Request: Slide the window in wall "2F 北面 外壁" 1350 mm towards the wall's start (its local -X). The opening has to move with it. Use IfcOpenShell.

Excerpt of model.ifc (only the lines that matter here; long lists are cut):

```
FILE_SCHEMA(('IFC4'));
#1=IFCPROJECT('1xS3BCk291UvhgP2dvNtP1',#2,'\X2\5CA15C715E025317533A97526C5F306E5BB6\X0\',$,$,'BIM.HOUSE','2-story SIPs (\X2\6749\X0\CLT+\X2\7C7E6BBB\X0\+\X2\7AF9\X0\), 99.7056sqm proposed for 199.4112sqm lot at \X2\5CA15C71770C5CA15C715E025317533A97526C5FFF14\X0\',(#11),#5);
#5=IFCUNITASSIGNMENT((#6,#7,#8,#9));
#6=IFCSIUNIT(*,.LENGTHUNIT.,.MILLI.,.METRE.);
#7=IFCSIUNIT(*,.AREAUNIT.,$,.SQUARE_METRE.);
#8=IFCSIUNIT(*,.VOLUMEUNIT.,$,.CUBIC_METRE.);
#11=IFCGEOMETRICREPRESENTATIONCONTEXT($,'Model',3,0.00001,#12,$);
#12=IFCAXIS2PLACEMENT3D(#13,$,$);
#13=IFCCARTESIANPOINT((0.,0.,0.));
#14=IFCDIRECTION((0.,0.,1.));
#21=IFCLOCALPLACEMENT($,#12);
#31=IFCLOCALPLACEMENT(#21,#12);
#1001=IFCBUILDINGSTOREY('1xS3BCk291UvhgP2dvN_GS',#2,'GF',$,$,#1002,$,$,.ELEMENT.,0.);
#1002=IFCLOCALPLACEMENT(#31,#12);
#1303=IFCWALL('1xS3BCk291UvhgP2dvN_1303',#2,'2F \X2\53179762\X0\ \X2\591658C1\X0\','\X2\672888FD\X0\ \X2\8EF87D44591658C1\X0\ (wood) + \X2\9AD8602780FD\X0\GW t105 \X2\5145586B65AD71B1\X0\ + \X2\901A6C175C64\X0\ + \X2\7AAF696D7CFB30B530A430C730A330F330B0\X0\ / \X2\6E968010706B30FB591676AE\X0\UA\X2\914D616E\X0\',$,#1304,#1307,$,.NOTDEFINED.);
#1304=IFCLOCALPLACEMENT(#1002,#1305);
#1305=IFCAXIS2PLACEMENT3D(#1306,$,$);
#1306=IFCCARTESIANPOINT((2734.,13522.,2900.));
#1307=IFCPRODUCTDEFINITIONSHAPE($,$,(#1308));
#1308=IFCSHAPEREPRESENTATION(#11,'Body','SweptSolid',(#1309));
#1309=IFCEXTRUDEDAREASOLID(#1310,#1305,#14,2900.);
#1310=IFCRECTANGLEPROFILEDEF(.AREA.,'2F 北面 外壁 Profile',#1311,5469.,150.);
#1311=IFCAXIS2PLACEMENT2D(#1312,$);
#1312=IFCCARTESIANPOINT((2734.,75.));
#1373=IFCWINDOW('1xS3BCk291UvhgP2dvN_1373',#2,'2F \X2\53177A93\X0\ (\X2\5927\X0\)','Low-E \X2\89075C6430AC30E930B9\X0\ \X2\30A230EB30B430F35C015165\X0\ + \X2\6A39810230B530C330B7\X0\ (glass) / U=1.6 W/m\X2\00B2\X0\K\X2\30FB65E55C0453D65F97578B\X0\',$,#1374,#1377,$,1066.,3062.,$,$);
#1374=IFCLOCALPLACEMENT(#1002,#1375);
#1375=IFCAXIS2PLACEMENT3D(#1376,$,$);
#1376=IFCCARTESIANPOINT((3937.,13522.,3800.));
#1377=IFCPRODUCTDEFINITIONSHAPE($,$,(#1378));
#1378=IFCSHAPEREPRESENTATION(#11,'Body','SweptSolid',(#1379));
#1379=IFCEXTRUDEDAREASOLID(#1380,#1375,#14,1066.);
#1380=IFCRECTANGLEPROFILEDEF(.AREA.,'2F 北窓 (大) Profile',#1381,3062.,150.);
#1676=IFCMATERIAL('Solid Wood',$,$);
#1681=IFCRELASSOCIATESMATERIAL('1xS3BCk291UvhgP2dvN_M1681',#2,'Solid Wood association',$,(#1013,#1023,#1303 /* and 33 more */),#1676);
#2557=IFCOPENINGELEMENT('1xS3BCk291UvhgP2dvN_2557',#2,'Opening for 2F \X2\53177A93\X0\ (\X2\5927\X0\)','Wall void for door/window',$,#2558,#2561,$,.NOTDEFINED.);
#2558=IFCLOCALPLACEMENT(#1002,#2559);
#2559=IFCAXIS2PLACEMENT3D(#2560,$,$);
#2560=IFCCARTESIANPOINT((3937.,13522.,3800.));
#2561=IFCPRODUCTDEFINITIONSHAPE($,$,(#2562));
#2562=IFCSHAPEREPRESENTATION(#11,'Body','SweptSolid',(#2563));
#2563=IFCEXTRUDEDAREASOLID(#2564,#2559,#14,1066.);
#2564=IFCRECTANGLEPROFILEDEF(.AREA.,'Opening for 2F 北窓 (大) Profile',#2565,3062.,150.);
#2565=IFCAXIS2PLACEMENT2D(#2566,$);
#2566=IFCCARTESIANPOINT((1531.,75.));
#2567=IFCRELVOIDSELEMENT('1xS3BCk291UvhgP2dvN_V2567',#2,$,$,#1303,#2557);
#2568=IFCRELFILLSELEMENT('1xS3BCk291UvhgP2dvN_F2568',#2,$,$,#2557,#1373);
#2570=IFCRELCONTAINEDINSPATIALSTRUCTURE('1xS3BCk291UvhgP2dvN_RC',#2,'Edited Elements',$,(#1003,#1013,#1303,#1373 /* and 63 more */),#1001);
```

```python
import ifcopenshell
import ifcopenshell.api.geometry
import ifcopenshell.util.placement

model = ifcopenshell.open("model.ifc")

window = model.by_guid("1xS3BCk291UvhgP2dvN_1373")
opening = window.FillsVoids[0].RelatingOpeningElement
wall = opening.VoidsElements[0].RelatingBuildingElement

wall_matrix = ifcopenshell.util.placement.get_local_placement(wall.ObjectPlacement)
shift = wall_matrix[:3, 0] * -1350.0
before = ifcopenshell.util.placement.get_local_placement(window.ObjectPlacement)[:3, 3].copy()

# The window is not placed relative to its opening, so move both.
for product in (opening, window):
    matrix = ifcopenshell.util.placement.get_local_placement(product.ObjectPlacement)
    matrix[:3, 3] += shift
    ifcopenshell.api.geometry.edit_object_placement(model, product=product, matrix=matrix, is_si=False)

after = ifcopenshell.util.placement.get_local_placement(window.ObjectPlacement)[:3, 3]
print("window moved by", (after - before).round(3) + 0.0)

model.write("model-out.ifc")
```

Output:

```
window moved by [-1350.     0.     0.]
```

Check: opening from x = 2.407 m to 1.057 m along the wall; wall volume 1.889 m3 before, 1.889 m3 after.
